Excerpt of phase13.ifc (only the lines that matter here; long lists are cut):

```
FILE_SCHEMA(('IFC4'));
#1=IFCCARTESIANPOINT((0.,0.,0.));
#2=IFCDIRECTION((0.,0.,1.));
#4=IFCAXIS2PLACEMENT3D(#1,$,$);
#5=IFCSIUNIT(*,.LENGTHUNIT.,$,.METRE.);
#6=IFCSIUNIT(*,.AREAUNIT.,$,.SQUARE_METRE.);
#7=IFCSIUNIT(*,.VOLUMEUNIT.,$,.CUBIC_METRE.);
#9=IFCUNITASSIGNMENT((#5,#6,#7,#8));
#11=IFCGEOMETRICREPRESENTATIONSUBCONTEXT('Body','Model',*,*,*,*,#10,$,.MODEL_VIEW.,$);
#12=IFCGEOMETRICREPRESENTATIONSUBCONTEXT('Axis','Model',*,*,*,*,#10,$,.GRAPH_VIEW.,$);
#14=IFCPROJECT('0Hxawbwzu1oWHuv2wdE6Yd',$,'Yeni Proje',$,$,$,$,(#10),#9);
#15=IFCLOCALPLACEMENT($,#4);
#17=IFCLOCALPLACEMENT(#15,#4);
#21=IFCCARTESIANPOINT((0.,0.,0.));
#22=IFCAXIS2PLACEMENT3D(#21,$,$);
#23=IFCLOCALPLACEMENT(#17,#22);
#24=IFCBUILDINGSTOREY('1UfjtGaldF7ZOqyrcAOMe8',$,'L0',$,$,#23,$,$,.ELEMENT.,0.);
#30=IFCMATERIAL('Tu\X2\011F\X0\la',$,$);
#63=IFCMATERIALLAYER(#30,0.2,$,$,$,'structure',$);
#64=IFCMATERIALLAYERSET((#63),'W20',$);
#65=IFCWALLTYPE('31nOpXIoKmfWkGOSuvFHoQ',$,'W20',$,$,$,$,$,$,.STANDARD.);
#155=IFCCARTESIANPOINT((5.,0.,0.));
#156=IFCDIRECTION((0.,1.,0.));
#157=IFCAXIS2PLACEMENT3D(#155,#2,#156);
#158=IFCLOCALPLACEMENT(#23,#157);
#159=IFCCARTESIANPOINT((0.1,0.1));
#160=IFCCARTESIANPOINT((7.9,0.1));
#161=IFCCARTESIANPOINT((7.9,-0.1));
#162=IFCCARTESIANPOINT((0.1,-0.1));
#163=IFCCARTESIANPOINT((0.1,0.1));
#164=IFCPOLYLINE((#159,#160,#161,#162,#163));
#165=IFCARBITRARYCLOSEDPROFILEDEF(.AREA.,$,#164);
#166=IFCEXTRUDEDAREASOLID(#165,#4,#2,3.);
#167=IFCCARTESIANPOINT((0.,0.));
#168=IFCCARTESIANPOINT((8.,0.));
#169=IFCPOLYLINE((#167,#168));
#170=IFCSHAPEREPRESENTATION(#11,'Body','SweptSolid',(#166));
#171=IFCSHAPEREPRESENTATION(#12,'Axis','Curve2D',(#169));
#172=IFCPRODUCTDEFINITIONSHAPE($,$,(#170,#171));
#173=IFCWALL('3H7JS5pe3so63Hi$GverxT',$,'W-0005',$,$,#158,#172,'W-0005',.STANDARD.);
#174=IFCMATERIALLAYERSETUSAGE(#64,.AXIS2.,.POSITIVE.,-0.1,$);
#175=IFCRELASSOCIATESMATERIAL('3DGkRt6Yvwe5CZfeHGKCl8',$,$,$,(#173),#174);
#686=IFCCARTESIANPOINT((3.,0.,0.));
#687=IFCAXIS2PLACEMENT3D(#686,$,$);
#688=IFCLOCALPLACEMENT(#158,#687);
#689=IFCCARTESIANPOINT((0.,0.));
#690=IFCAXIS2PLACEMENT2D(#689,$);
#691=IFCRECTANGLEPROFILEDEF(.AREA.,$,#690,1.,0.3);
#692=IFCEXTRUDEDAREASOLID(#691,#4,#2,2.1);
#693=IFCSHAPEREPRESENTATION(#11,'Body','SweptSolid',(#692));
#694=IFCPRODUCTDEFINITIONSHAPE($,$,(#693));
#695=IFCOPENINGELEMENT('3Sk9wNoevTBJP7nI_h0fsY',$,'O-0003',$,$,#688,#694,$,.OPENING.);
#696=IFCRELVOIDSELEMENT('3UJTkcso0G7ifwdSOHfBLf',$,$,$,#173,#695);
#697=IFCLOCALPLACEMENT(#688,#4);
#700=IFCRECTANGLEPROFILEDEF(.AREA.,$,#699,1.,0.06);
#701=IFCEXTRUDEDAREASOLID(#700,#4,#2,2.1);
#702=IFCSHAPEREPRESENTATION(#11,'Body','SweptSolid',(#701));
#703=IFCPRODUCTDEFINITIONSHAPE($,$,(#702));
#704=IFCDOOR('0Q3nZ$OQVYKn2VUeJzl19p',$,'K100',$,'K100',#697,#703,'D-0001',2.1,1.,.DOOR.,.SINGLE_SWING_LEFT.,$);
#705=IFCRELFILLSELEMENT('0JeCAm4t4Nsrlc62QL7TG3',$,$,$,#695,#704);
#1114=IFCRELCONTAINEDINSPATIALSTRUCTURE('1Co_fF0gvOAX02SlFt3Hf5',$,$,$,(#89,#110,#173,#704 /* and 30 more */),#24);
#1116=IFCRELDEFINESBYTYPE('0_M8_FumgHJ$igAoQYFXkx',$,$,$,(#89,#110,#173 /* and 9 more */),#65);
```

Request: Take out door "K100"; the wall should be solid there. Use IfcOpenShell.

```python
import ifcopenshell
import ifcopenshell.api.feature
import ifcopenshell.api.root
import ifcopenshell.geom
import ifcopenshell.util.shape

model = ifcopenshell.open("phase13.ifc")
settings = ifcopenshell.geom.settings()


def volume(element):
    """Net volume in cubic metres, openings subtracted."""
    shape = ifcopenshell.geom.create_shape(settings, element)
    return ifcopenshell.util.shape.get_volume(shape.geometry)


door = model.by_guid("0Q3nZ$OQVYKn2VUeJzl19p")
opening = door.FillsVoids[0].RelatingOpeningElement
wall = opening.VoidsElements[0].RelatingBuildingElement
before = volume(wall)

ifcopenshell.api.root.remove_product(model, product=door)
ifcopenshell.api.feature.remove_feature(model, feature=opening)

after = volume(wall)

print(f"wall volume {before:.3f} -> {after:.3f} m3")

model.write("phase13_v2.ifc")
```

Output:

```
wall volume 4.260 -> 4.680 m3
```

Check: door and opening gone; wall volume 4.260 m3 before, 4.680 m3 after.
